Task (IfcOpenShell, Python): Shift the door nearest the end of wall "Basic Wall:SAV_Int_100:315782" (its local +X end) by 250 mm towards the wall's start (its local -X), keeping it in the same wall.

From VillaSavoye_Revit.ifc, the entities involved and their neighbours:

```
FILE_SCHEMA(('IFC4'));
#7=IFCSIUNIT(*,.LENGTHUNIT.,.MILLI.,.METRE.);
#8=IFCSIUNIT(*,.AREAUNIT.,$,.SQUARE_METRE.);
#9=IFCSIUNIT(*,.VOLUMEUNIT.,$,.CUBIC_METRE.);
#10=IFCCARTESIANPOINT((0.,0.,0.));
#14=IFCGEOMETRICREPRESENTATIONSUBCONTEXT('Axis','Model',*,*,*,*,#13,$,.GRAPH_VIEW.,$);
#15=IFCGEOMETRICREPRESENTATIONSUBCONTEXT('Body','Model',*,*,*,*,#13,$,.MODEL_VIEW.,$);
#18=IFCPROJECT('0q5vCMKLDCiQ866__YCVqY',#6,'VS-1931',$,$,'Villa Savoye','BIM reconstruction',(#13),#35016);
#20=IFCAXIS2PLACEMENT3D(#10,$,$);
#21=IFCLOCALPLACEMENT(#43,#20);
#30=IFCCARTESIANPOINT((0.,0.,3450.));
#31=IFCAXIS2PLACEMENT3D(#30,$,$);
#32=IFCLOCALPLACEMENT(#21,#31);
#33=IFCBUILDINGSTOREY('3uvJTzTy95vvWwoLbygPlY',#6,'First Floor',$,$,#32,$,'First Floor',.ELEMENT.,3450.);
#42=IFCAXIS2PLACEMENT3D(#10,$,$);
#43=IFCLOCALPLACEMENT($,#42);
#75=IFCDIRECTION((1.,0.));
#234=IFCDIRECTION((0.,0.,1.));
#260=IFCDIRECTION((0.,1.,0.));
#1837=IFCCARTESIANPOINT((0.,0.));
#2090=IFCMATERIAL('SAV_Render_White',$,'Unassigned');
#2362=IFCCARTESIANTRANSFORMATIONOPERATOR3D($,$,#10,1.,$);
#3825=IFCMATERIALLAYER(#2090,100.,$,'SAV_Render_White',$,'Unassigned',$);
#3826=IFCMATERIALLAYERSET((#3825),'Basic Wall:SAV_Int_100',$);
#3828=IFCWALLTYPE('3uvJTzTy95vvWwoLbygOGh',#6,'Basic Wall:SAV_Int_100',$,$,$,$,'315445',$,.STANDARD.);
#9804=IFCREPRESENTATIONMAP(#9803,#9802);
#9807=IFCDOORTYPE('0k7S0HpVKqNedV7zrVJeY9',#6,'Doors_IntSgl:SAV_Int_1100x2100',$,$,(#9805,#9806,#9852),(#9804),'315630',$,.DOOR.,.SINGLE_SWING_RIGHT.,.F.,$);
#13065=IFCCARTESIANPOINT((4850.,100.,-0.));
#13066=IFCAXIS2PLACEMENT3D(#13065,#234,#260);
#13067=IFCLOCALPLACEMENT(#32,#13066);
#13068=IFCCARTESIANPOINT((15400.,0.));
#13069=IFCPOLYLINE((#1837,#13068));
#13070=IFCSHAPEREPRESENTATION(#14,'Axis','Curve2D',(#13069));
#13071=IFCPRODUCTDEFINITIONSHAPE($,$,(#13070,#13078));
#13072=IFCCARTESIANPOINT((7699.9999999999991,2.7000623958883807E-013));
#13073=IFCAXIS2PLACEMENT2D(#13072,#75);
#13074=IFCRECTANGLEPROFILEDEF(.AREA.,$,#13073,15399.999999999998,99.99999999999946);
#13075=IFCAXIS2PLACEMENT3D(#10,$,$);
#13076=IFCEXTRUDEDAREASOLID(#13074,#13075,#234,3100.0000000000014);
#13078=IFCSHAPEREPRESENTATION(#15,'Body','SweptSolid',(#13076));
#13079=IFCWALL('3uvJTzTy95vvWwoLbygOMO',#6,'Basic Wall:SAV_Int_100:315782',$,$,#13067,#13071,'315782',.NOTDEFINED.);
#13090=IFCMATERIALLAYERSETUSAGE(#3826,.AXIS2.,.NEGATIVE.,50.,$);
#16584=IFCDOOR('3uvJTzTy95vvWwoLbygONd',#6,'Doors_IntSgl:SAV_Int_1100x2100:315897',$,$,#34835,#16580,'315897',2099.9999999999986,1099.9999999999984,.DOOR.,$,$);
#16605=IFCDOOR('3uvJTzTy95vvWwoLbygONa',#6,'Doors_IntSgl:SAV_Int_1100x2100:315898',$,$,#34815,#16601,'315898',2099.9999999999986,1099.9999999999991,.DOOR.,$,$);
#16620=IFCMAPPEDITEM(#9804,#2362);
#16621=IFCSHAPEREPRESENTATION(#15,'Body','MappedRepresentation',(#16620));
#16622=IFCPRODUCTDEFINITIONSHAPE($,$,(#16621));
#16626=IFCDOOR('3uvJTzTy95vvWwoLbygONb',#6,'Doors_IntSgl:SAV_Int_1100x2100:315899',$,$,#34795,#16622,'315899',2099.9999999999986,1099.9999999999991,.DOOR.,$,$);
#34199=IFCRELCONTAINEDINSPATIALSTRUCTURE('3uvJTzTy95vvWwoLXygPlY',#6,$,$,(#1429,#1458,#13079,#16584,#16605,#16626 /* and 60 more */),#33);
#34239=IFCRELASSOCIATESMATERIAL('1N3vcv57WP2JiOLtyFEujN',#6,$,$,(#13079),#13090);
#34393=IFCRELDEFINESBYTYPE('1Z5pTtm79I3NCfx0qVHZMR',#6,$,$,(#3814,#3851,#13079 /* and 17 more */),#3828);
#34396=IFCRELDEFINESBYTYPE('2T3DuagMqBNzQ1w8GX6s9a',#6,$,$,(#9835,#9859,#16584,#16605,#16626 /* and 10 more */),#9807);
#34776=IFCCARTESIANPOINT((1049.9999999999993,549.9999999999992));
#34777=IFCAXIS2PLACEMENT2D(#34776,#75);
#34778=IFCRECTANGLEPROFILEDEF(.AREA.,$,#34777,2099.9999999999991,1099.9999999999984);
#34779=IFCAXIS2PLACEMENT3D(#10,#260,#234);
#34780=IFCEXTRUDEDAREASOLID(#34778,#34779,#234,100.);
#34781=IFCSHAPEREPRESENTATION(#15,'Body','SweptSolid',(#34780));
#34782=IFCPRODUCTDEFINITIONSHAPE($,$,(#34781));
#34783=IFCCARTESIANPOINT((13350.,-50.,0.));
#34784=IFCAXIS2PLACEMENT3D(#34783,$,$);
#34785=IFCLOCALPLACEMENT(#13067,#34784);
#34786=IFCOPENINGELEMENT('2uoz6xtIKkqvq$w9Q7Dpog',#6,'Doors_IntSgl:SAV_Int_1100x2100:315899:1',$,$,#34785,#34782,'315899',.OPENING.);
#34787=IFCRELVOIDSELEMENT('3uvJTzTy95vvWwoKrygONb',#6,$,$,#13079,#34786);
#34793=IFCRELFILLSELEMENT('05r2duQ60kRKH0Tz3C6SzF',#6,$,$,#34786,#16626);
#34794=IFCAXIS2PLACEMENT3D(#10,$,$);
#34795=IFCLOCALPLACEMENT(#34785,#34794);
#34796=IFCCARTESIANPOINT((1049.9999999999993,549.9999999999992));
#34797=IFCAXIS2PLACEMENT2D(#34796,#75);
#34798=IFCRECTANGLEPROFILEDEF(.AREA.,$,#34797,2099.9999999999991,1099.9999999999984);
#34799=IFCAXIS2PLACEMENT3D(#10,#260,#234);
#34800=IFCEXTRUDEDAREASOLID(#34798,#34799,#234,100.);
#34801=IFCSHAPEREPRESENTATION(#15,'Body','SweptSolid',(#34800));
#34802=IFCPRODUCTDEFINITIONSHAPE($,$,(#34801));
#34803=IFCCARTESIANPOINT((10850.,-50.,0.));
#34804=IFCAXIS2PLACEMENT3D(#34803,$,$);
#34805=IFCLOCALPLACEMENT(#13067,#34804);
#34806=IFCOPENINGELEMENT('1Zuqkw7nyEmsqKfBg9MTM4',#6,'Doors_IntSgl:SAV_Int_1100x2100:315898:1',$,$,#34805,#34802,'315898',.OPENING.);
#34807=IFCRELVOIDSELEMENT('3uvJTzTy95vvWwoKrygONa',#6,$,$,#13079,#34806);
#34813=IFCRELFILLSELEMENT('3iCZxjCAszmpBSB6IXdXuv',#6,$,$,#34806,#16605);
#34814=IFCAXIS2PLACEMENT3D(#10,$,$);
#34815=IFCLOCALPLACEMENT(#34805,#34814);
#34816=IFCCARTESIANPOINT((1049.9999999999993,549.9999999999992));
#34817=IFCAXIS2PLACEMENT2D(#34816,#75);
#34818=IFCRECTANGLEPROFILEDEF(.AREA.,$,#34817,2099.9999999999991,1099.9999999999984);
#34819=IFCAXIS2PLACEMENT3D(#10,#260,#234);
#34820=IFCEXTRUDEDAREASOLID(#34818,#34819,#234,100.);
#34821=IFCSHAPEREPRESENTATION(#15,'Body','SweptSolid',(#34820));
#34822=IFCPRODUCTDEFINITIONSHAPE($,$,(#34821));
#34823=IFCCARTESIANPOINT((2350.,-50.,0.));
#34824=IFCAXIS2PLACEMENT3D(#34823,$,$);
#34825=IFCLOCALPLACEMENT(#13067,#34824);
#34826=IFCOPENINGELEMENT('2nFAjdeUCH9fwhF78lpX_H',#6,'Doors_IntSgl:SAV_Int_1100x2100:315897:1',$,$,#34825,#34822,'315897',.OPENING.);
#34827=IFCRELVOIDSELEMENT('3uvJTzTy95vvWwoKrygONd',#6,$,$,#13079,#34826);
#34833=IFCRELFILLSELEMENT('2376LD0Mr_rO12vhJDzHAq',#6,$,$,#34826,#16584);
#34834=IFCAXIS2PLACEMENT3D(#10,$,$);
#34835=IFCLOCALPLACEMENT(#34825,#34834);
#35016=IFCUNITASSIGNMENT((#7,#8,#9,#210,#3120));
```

```python
import ifcopenshell
import ifcopenshell.api.geometry
import ifcopenshell.util.placement
import ifcopenshell.util.unit

model = ifcopenshell.open("VillaSavoye_Revit.ifc")
unit_scale = ifcopenshell.util.unit.calculate_unit_scale(model)

door = model.by_guid("3uvJTzTy95vvWwoLbygONb")
opening = door.FillsVoids[0].RelatingOpeningElement
wall = opening.VoidsElements[0].RelatingBuildingElement

wall_matrix = ifcopenshell.util.placement.get_local_placement(wall.ObjectPlacement)
shift = wall_matrix[:3, 0] * -0.25 / unit_scale
before = ifcopenshell.util.placement.get_local_placement(door.ObjectPlacement)[:3, 3].copy()

# The door is placed relative to its opening, so it follows when the opening moves.
matrix = ifcopenshell.util.placement.get_local_placement(opening.ObjectPlacement)
matrix[:3, 3] += shift
ifcopenshell.api.geometry.edit_object_placement(
    model, product=opening, matrix=matrix, is_si=False, should_transform_children=True
)

after = ifcopenshell.util.placement.get_local_placement(door.ObjectPlacement)[:3, 3]
print("door moved by", (after - before).round(3) + 0.0)

model.write("VillaSavoye_Revit_rev.ifc")
```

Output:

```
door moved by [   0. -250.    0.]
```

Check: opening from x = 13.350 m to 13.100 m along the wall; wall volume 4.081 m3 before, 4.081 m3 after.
